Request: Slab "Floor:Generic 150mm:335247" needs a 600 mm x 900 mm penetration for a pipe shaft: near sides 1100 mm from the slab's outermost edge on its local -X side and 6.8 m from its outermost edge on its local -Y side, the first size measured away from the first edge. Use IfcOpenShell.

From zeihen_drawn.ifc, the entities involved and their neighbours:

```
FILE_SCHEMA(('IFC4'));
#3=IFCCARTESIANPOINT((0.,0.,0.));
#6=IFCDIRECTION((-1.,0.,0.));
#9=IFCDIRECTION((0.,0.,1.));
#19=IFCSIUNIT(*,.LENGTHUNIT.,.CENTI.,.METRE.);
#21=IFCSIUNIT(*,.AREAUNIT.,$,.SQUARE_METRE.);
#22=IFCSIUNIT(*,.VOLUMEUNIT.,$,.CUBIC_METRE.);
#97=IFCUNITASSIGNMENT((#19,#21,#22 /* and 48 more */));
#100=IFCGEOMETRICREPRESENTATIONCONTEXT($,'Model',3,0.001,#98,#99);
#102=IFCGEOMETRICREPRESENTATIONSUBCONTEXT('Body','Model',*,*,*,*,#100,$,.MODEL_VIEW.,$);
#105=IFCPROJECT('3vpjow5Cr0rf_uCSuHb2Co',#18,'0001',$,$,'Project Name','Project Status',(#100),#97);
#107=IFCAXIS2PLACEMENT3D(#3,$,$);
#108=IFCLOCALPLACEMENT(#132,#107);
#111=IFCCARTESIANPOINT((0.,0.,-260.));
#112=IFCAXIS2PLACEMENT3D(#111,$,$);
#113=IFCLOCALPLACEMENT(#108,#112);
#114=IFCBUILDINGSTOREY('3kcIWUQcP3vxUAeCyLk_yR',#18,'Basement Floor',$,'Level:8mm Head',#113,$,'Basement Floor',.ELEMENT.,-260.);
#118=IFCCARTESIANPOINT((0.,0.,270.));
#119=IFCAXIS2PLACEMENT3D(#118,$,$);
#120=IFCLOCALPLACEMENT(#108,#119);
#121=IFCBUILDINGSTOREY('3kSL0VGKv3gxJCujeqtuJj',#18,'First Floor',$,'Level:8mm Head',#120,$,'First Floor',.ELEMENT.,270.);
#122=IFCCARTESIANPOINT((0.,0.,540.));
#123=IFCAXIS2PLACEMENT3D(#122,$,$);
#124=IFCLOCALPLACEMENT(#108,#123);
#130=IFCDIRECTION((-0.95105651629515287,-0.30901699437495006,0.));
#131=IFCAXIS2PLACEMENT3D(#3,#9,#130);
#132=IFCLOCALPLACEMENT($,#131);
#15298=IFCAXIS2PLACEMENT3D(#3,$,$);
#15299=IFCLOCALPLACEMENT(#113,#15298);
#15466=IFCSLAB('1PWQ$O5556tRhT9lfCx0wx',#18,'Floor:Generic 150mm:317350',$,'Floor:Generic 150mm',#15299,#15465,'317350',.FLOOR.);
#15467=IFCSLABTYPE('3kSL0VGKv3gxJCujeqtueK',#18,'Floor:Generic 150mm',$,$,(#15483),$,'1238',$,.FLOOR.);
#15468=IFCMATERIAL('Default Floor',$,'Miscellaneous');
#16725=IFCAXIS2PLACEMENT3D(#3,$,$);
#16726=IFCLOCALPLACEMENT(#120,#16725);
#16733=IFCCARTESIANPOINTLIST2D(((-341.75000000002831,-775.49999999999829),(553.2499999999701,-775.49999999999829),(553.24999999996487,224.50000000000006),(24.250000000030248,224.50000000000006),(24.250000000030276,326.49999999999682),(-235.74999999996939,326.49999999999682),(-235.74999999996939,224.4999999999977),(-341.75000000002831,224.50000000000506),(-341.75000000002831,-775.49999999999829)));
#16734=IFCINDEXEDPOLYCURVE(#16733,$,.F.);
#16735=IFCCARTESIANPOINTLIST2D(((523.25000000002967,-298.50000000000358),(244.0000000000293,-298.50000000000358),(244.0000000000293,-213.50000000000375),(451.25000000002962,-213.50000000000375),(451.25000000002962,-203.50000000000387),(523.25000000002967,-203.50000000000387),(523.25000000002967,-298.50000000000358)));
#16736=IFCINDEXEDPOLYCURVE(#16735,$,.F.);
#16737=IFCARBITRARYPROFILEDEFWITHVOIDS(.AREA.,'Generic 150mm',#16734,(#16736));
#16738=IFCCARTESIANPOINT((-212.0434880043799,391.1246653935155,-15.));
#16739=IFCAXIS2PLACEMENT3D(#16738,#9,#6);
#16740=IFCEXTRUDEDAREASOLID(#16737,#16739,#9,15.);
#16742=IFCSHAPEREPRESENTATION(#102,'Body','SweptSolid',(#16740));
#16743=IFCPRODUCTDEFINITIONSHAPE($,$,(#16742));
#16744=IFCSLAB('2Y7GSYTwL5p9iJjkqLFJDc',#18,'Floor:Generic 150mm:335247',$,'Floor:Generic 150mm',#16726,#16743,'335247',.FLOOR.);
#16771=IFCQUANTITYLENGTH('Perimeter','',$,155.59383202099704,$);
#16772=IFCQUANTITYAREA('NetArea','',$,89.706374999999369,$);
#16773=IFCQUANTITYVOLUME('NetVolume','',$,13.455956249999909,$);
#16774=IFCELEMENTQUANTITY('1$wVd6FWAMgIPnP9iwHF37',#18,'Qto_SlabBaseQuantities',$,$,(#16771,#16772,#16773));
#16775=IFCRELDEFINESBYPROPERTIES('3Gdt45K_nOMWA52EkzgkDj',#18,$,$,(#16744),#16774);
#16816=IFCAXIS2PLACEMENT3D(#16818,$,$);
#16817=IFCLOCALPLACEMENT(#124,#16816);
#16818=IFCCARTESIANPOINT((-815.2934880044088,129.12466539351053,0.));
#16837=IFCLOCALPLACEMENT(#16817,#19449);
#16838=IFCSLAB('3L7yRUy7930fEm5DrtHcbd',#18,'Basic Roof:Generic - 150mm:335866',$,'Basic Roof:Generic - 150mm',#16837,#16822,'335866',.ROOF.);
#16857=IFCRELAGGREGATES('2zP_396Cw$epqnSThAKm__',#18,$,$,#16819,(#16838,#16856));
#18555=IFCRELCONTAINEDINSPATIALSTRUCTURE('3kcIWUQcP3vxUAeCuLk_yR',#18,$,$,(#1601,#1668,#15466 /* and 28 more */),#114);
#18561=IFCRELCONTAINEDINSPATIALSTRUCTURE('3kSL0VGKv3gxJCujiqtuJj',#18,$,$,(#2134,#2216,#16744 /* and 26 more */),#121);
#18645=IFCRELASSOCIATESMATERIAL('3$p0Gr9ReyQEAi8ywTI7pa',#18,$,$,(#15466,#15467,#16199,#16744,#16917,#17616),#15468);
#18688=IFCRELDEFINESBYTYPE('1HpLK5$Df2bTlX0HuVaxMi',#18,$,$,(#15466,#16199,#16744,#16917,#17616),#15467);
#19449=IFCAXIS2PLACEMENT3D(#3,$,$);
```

```python
import numpy as np
import ifcopenshell
import ifcopenshell.api.feature
import ifcopenshell.api.geometry
import ifcopenshell.api.pset
import ifcopenshell.api.root
import ifcopenshell.geom
import ifcopenshell.util.element
import ifcopenshell.util.placement
import ifcopenshell.util.representation
import ifcopenshell.util.shape
import ifcopenshell.util.unit

model = ifcopenshell.open("zeihen_drawn.ifc")
unit_scale = ifcopenshell.util.unit.calculate_unit_scale(model)
area_scale = ifcopenshell.util.unit.calculate_unit_scale(model, "AREAUNIT")
volume_scale = ifcopenshell.util.unit.calculate_unit_scale(model, "VOLUMEUNIT")
settings = ifcopenshell.geom.settings()


def volume(element):
    """Net volume in cubic metres, openings subtracted."""
    shape = ifcopenshell.geom.create_shape(settings, element)
    return ifcopenshell.util.shape.get_volume(shape.geometry)


slab = model.by_guid("2Y7GSYTwL5p9iJjkqLFJDc")
before = volume(slab)

# Extent in the slab's own axes, in metres. The edges named are its -X and -Y sides.
slab_shape = ifcopenshell.geom.create_shape(settings, slab)
vertices = ifcopenshell.util.shape.get_vertices(slab_shape.geometry)
x_min, y_min, bottom = vertices.min(axis=0)
top = vertices[:, 2].max()

opening = ifcopenshell.api.root.create_entity(model, ifc_class="IfcOpeningElement", name="Pipe shaft opening", predefined_type="OPENING")
context = ifcopenshell.util.representation.get_context(model, "Model", "Body", "MODEL_VIEW")
width, depth = 0.6, 0.9
outline = [(0.0, 0.0), (width, 0.0), (width, depth), (0.0, depth), (0.0, 0.0)]
# Overshoot both faces by 50 mm so the cut is clean.
shape = ifcopenshell.api.geometry.add_slab_representation(
    model, context=context, depth=top - bottom + 0.1, polyline=outline
)
ifcopenshell.api.geometry.assign_representation(model, product=opening, representation=shape)

matrix = ifcopenshell.util.placement.get_local_placement(slab.ObjectPlacement)
matrix[:, 3] = matrix @ np.append(np.array([x_min + 1.1, y_min + 6.8, bottom - 0.05]) / unit_scale, 1.0)
ifcopenshell.api.geometry.edit_object_placement(model, product=opening, matrix=matrix, is_si=False)
ifcopenshell.api.feature.add_feature(model, feature=opening, element=slab)

after = volume(slab)

# Update the slab's stored quantities.
qto = model.by_id(ifcopenshell.util.element.get_pset(slab, "Qto_SlabBaseQuantities", should_inherit=False)["id"])
ifcopenshell.api.pset.edit_qto(model, qto=qto, properties={
    "NetArea": after / (top - bottom) / area_scale,
    "NetVolume": after / volume_scale,
})

print(f"slab volume {before:.3f} -> {after:.3f} m3")

model.write("zeihen_drawn_rev.ifc")
```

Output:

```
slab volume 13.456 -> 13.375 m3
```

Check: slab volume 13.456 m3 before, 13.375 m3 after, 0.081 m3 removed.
